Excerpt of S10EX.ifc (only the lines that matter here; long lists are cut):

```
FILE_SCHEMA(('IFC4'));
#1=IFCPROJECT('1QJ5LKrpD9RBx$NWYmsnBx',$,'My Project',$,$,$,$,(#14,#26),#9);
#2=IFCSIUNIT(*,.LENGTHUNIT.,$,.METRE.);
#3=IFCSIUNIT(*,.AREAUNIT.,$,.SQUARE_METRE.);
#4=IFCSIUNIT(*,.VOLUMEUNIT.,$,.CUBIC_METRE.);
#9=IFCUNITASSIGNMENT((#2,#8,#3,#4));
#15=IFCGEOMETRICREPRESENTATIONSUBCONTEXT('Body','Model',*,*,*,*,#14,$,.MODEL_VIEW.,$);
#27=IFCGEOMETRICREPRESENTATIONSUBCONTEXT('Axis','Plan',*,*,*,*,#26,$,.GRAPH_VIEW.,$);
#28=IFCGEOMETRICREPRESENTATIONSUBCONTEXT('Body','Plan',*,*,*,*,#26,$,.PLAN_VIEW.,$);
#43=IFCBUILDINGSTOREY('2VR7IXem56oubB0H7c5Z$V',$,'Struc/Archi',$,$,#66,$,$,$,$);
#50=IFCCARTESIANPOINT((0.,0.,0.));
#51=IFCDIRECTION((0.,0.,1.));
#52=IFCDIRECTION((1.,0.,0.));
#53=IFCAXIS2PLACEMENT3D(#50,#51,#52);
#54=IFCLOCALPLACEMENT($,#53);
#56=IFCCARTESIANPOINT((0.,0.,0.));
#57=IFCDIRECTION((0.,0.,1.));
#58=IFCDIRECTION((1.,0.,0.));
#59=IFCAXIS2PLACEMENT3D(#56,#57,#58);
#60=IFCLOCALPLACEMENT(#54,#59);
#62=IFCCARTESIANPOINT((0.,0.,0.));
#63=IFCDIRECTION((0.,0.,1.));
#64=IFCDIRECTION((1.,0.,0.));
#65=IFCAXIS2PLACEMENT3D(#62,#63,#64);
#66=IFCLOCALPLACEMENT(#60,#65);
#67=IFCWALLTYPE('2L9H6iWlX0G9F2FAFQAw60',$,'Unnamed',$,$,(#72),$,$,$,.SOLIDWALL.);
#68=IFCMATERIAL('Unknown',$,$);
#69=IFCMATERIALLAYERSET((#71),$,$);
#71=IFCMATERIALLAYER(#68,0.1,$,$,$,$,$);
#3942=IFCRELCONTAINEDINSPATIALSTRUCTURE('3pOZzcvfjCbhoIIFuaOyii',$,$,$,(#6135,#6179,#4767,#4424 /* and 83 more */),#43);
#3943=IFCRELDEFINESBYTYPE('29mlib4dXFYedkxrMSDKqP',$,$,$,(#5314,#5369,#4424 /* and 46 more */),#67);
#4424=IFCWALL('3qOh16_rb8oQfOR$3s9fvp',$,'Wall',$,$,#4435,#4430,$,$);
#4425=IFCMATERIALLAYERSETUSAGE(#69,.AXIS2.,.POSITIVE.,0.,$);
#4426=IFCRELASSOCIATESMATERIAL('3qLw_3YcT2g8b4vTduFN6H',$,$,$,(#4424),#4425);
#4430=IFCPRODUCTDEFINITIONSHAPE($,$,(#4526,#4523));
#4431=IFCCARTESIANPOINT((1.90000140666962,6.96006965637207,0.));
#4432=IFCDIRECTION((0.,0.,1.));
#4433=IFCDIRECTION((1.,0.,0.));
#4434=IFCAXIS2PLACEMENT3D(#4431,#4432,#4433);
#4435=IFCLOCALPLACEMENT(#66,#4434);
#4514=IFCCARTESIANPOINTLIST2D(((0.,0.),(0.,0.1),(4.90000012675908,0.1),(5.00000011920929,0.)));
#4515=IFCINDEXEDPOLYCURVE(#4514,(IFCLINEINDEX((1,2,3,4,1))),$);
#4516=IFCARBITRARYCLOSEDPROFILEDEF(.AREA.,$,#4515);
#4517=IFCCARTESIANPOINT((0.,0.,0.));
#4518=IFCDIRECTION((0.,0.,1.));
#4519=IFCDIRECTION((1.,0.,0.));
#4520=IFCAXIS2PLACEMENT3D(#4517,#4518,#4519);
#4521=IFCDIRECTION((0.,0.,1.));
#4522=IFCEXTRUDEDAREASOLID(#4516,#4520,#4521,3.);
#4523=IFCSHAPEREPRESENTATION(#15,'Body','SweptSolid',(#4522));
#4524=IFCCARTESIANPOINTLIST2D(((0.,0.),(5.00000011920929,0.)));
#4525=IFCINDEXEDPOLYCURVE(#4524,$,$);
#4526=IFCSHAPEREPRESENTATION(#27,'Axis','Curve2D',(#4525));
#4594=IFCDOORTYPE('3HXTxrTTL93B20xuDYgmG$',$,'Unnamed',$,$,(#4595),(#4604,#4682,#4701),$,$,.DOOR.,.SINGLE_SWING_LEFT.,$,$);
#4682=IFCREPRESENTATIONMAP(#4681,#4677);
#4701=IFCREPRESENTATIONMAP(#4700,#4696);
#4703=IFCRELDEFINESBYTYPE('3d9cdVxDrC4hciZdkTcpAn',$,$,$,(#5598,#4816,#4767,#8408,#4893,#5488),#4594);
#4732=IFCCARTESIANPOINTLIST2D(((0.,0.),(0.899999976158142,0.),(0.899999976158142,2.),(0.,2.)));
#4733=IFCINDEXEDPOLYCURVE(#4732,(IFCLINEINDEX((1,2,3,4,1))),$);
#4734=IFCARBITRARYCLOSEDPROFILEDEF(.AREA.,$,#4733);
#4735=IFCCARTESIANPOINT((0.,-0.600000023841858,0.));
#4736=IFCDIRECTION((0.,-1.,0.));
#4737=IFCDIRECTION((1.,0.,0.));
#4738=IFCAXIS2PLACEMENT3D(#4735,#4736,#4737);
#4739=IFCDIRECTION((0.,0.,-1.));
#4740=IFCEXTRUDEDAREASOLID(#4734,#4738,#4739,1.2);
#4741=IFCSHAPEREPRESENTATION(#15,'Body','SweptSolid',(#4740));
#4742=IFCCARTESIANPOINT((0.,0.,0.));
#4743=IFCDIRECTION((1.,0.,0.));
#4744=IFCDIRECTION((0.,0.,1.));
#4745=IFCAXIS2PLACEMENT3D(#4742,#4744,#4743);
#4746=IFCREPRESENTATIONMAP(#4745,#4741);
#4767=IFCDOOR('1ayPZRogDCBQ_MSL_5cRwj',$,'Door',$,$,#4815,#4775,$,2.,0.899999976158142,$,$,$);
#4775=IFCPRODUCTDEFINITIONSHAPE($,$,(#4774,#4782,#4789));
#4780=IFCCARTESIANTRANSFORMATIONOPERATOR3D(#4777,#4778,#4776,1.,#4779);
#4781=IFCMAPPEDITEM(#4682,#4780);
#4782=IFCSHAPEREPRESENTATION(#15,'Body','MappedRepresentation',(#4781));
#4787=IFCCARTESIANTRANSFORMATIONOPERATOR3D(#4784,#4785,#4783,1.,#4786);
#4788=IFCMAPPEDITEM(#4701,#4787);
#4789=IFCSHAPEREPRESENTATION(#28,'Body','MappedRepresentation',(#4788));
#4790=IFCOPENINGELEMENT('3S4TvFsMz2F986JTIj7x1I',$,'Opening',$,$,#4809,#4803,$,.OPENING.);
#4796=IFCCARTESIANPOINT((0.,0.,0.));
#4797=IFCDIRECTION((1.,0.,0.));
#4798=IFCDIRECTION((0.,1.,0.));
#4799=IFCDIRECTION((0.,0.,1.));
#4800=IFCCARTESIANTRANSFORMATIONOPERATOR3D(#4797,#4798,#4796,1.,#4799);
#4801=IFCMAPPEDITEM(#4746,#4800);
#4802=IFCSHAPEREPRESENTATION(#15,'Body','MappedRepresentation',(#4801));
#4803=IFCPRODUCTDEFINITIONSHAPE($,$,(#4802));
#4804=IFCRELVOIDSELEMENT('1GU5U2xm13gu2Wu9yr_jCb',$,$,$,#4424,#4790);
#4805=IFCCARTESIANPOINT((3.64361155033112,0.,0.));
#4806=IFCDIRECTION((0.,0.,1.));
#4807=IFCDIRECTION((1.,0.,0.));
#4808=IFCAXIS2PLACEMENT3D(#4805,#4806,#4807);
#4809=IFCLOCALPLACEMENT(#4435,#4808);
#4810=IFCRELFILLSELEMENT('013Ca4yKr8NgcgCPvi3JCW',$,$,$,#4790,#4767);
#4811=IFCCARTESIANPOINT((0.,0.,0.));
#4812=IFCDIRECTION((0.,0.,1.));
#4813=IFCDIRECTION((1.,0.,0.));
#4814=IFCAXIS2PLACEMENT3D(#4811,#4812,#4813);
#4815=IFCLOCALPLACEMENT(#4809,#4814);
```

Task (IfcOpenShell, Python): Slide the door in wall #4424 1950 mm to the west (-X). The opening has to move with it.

```python
import ifcopenshell
import ifcopenshell.api.geometry
import ifcopenshell.util.placement
import ifcopenshell.util.unit

model = ifcopenshell.open("S10EX.ifc")
unit_scale = ifcopenshell.util.unit.calculate_unit_scale(model)

door = model.by_guid("1ayPZRogDCBQ_MSL_5cRwj")
opening = door.FillsVoids[0].RelatingOpeningElement
wall = opening.VoidsElements[0].RelatingBuildingElement

wall_matrix = ifcopenshell.util.placement.get_local_placement(wall.ObjectPlacement)
shift = wall_matrix[:3, 0] * -1.95 / unit_scale
before = ifcopenshell.util.placement.get_local_placement(door.ObjectPlacement)[:3, 3].copy()

# The door is placed relative to its opening, so it follows when the opening moves.
matrix = ifcopenshell.util.placement.get_local_placement(opening.ObjectPlacement)
matrix[:3, 3] += shift
ifcopenshell.api.geometry.edit_object_placement(
    model, product=opening, matrix=matrix, is_si=False, should_transform_children=True
)

after = ifcopenshell.util.placement.get_local_placement(door.ObjectPlacement)[:3, 3]
print("door moved by", (after - before).round(3) + 0.0)

model.write("S10EX_edited.ifc")
```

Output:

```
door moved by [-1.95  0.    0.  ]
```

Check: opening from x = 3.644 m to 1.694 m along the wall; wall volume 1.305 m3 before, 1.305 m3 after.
